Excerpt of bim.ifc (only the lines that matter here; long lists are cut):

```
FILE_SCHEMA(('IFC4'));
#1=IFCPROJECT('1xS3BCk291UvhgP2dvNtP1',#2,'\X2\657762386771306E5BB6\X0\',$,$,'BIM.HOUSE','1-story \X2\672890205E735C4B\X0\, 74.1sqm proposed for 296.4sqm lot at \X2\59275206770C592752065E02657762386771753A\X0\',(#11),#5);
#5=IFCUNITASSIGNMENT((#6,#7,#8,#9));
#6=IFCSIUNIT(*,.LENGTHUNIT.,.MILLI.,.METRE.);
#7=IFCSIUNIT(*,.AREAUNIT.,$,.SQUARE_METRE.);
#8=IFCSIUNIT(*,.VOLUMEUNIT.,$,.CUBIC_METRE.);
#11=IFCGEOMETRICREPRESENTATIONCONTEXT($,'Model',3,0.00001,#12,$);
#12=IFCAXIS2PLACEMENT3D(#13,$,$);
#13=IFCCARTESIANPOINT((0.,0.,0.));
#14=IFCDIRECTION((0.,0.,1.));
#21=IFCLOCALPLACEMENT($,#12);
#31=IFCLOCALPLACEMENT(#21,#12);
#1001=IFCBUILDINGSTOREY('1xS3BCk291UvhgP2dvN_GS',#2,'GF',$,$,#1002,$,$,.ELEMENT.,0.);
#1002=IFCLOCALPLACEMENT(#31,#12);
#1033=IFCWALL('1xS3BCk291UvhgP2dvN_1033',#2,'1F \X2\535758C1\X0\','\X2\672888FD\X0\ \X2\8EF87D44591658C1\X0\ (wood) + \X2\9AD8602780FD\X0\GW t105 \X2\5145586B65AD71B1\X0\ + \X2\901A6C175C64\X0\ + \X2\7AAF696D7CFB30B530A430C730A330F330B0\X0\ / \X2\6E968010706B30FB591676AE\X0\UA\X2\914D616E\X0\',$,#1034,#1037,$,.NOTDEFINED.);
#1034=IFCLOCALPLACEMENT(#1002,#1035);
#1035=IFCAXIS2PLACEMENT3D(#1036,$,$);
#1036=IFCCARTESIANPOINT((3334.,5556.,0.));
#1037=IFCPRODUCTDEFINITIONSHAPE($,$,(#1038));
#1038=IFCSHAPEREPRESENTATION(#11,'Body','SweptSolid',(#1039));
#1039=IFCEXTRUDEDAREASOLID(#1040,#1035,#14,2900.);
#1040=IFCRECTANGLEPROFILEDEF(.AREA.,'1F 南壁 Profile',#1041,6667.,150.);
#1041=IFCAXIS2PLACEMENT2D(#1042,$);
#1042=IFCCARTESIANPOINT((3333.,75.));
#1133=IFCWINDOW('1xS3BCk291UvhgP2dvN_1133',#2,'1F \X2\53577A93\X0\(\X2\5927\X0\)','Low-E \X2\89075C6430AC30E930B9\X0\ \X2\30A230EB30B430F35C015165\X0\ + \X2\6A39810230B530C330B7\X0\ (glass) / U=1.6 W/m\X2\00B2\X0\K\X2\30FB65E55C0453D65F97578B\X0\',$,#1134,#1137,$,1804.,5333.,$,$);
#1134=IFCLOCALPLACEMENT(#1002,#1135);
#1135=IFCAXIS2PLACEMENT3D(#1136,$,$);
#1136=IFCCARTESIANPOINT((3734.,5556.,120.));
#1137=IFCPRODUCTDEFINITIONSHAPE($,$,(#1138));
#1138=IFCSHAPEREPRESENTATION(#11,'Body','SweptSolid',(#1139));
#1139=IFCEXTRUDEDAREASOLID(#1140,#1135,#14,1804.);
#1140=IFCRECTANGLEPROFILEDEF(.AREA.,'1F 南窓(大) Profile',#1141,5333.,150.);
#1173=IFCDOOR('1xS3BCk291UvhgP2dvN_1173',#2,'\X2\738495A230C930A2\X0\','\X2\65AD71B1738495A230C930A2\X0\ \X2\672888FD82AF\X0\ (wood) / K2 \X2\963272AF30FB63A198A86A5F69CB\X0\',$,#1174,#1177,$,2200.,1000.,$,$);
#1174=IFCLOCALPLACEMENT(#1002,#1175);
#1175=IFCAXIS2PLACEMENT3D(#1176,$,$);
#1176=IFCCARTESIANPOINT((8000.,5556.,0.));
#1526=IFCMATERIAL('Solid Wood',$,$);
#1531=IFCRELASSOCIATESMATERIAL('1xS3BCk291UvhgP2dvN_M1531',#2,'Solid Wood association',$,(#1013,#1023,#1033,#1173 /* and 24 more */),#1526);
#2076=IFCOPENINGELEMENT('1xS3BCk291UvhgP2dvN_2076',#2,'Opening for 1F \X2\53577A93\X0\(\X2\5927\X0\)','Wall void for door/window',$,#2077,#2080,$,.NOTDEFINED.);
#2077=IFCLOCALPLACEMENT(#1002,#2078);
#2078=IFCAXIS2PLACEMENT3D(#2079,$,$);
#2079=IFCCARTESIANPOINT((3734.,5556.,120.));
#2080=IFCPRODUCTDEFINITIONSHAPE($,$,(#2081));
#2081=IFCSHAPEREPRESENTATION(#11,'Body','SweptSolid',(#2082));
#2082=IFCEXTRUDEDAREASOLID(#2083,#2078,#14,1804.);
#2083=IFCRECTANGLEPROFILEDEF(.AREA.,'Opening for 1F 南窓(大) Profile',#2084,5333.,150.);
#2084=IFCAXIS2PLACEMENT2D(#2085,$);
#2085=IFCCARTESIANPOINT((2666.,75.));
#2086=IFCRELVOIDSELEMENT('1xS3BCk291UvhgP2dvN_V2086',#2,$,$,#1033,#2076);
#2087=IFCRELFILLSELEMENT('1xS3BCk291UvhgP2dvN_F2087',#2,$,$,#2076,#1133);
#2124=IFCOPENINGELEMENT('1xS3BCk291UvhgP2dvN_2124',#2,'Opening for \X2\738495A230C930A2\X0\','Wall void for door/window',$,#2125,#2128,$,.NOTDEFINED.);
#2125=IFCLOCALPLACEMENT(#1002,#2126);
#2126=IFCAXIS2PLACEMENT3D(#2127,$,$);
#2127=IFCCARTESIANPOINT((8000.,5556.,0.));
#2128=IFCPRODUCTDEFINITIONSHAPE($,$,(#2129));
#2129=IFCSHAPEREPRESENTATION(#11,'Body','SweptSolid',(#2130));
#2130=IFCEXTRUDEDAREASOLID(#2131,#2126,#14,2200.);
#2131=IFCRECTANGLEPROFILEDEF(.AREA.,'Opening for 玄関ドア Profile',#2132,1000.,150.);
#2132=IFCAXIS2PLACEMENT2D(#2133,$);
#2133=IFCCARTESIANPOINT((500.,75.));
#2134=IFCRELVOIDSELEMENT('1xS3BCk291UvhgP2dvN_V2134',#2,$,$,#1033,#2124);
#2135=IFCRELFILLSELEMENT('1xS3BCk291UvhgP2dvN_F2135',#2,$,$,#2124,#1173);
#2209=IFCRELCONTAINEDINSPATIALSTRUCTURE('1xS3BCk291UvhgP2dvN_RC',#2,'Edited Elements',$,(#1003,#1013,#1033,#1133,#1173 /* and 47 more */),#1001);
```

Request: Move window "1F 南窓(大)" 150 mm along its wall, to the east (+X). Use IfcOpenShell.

```python
import ifcopenshell
import ifcopenshell.api.geometry
import ifcopenshell.util.placement
import ifcopenshell.util.unit

model = ifcopenshell.open("bim.ifc")
unit_scale = ifcopenshell.util.unit.calculate_unit_scale(model)

window = model.by_guid("1xS3BCk291UvhgP2dvN_1133")
opening = window.FillsVoids[0].RelatingOpeningElement
wall = opening.VoidsElements[0].RelatingBuildingElement

wall_matrix = ifcopenshell.util.placement.get_local_placement(wall.ObjectPlacement)
shift = wall_matrix[:3, 0] * 0.15 / unit_scale
before = ifcopenshell.util.placement.get_local_placement(window.ObjectPlacement)[:3, 3].copy()

# The window is not placed relative to its opening, so move both.
for product in (opening, window):
    matrix = ifcopenshell.util.placement.get_local_placement(product.ObjectPlacement)
    matrix[:3, 3] += shift
    ifcopenshell.api.geometry.edit_object_placement(model, product=product, matrix=matrix, is_si=False)

after = ifcopenshell.util.placement.get_local_placement(window.ObjectPlacement)[:3, 3]
print("window moved by", (after - before).round(3) + 0.0)

model.write("bim_updated.ifc")
```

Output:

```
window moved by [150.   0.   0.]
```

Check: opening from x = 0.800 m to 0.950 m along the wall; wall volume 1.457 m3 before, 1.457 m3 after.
